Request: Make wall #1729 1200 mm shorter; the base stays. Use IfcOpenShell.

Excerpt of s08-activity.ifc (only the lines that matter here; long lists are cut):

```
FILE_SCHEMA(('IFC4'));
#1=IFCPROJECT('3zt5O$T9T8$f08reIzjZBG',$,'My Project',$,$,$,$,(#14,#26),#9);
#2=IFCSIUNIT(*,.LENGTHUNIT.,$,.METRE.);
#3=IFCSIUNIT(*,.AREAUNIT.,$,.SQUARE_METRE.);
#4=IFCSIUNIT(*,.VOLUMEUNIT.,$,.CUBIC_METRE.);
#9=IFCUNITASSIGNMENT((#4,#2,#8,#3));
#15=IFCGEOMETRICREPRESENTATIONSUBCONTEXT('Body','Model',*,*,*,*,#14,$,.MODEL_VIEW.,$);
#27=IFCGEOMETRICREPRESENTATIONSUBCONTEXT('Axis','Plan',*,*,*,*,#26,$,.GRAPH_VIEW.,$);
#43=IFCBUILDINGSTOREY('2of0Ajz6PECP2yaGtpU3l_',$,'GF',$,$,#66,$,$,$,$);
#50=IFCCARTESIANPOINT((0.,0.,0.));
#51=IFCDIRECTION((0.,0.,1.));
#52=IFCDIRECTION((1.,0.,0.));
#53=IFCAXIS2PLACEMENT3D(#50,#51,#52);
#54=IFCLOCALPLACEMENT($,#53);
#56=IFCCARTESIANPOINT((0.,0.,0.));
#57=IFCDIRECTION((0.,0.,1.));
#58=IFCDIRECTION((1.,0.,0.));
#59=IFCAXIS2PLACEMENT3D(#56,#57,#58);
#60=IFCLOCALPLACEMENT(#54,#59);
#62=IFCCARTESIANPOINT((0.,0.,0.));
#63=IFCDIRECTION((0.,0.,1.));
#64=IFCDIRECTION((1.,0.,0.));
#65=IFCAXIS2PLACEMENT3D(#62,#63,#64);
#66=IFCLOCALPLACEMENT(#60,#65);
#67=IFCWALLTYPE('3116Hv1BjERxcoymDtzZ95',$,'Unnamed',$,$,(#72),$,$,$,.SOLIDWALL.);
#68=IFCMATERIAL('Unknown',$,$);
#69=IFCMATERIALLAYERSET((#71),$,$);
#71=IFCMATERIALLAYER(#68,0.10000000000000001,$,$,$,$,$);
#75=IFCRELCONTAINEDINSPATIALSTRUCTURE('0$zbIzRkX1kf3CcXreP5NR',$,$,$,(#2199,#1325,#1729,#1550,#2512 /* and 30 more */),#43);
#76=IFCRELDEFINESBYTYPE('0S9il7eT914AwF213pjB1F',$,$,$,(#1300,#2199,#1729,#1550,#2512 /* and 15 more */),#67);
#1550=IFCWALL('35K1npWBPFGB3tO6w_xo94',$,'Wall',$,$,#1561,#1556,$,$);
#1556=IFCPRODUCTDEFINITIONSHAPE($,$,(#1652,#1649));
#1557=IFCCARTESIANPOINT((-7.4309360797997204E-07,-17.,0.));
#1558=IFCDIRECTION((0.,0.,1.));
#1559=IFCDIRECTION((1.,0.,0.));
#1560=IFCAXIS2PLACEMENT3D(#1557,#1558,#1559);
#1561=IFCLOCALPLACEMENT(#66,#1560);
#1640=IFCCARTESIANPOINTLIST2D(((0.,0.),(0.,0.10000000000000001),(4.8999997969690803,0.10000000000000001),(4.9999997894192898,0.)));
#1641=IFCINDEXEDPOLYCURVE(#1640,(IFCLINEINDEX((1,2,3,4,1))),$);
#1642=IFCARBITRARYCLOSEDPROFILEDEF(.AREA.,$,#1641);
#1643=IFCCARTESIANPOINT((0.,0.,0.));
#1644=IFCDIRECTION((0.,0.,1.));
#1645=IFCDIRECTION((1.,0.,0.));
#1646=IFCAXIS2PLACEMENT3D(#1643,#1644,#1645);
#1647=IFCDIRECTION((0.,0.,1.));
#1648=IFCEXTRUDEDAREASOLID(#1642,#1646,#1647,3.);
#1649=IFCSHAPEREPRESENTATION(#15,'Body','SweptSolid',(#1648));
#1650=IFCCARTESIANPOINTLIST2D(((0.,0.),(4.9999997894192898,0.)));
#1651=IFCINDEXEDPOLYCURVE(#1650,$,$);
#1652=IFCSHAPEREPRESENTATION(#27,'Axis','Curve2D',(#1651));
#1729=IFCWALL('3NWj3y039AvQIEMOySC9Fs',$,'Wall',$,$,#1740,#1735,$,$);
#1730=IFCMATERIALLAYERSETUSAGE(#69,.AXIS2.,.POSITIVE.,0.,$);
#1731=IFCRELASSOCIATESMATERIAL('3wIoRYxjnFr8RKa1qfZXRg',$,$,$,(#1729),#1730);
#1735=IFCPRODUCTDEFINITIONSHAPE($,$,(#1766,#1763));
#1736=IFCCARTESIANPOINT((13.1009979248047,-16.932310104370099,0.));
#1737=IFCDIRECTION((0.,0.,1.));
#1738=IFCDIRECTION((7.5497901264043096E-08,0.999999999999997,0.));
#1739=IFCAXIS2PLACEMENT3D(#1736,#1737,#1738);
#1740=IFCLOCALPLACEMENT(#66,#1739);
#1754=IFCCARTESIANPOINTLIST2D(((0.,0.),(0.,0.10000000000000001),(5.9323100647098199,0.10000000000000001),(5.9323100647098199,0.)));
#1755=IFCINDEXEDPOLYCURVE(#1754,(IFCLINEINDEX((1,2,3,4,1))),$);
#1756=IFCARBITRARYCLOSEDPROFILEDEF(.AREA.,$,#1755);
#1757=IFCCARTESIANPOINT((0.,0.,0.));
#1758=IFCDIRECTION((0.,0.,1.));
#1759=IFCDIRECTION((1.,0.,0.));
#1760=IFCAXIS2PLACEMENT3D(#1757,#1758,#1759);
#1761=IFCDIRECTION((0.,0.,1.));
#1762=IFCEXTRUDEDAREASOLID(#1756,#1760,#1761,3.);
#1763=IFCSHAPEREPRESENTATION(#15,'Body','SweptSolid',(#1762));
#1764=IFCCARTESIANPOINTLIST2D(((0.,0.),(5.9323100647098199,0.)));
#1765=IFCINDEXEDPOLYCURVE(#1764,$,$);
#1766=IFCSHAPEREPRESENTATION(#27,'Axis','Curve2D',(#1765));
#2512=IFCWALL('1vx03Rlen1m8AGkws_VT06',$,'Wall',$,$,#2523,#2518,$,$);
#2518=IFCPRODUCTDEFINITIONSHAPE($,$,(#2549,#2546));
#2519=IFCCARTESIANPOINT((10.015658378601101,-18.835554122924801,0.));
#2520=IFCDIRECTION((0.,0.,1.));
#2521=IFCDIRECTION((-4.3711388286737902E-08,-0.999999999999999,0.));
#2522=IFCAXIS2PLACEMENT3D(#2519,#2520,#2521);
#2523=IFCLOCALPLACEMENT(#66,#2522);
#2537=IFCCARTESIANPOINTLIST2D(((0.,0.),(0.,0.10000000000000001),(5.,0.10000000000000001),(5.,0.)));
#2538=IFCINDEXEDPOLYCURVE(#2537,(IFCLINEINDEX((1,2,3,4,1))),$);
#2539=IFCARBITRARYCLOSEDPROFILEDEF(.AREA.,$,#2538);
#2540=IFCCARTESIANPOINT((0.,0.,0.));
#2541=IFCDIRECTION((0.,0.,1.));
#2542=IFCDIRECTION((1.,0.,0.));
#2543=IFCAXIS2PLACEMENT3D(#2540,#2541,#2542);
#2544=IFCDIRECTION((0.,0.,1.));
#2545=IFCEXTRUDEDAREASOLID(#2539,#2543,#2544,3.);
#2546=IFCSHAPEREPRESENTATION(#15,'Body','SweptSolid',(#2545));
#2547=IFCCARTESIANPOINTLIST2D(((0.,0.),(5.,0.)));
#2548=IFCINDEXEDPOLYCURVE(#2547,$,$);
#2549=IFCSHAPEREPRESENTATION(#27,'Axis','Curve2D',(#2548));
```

```python
import ifcopenshell
import ifcopenshell.geom
import ifcopenshell.util.representation
import ifcopenshell.util.shape

model = ifcopenshell.open("s08-activity.ifc")
settings = ifcopenshell.geom.settings()


def volume(element):
    """Net volume in cubic metres, openings subtracted."""
    shape = ifcopenshell.geom.create_shape(settings, element)
    return ifcopenshell.util.shape.get_volume(shape.geometry)


wall = model.by_guid("3NWj3y039AvQIEMOySC9Fs")
before = volume(wall)

body = ifcopenshell.util.representation.get_representation(wall, "Model", "Body")
solid = body.Items[0]
old_height = solid.Depth
solid.Depth -= 1.2
after = volume(wall)

print(f"height {old_height:g} -> {solid.Depth:g}, volume {before:.3f} -> {after:.3f} m3")

model.write("s08-activity_v2.ifc")
```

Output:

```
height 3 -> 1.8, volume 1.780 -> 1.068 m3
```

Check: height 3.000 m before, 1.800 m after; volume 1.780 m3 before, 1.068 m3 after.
